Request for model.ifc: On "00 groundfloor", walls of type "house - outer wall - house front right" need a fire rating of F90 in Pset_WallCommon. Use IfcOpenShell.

First a look at what the model holds.

```python
import ifcopenshell
import ifcopenshell.util.element

model = ifcopenshell.open("model.ifc")
print(model.schema)
storey = next(s for s in model.by_type("IfcBuildingStorey") if s.Name == "00 groundfloor")
walls = [e for e in ifcopenshell.util.element.get_decomposition(storey) if e.is_a("IfcWall")]
seen = {}
for e in walls:
    element_type = ifcopenshell.util.element.get_type(e)
    key = (element_type.Name if element_type != e and element_type else None, ifcopenshell.util.element.get_pset(e, "Pset_WallCommon", "FireRating"))
    seen[key] = seen.get(key, 0) + 1
for (name, value), count in sorted(seen.items(), key=str):
    print(count, "x", name, "|", value)
```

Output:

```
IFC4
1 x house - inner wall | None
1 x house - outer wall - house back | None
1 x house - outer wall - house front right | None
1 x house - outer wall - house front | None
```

```python
import ifcopenshell
import ifcopenshell.api.pset
import ifcopenshell.util.element

model = ifcopenshell.open("model.ifc")

storey = next(s for s in model.by_type("IfcBuildingStorey") if s.Name == "00 groundfloor")
walls = [e for e in ifcopenshell.util.element.get_decomposition(storey) if e.is_a("IfcWall")]

count = 0
for e in walls:
    element_type = ifcopenshell.util.element.get_type(e)
    if element_type in (None, e) or element_type.Name != "house - outer wall - house front right":
        continue
    # add_pset returns the element's existing set when there is one.
    pset = ifcopenshell.api.pset.add_pset(model, product=e, name="Pset_WallCommon")
    ifcopenshell.api.pset.edit_pset(model, pset=pset, properties={"FireRating": "F90"})
    count += 1

print(count, "walls updated")

model.write("model_edited.ifc")
```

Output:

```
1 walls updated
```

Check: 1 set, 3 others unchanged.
